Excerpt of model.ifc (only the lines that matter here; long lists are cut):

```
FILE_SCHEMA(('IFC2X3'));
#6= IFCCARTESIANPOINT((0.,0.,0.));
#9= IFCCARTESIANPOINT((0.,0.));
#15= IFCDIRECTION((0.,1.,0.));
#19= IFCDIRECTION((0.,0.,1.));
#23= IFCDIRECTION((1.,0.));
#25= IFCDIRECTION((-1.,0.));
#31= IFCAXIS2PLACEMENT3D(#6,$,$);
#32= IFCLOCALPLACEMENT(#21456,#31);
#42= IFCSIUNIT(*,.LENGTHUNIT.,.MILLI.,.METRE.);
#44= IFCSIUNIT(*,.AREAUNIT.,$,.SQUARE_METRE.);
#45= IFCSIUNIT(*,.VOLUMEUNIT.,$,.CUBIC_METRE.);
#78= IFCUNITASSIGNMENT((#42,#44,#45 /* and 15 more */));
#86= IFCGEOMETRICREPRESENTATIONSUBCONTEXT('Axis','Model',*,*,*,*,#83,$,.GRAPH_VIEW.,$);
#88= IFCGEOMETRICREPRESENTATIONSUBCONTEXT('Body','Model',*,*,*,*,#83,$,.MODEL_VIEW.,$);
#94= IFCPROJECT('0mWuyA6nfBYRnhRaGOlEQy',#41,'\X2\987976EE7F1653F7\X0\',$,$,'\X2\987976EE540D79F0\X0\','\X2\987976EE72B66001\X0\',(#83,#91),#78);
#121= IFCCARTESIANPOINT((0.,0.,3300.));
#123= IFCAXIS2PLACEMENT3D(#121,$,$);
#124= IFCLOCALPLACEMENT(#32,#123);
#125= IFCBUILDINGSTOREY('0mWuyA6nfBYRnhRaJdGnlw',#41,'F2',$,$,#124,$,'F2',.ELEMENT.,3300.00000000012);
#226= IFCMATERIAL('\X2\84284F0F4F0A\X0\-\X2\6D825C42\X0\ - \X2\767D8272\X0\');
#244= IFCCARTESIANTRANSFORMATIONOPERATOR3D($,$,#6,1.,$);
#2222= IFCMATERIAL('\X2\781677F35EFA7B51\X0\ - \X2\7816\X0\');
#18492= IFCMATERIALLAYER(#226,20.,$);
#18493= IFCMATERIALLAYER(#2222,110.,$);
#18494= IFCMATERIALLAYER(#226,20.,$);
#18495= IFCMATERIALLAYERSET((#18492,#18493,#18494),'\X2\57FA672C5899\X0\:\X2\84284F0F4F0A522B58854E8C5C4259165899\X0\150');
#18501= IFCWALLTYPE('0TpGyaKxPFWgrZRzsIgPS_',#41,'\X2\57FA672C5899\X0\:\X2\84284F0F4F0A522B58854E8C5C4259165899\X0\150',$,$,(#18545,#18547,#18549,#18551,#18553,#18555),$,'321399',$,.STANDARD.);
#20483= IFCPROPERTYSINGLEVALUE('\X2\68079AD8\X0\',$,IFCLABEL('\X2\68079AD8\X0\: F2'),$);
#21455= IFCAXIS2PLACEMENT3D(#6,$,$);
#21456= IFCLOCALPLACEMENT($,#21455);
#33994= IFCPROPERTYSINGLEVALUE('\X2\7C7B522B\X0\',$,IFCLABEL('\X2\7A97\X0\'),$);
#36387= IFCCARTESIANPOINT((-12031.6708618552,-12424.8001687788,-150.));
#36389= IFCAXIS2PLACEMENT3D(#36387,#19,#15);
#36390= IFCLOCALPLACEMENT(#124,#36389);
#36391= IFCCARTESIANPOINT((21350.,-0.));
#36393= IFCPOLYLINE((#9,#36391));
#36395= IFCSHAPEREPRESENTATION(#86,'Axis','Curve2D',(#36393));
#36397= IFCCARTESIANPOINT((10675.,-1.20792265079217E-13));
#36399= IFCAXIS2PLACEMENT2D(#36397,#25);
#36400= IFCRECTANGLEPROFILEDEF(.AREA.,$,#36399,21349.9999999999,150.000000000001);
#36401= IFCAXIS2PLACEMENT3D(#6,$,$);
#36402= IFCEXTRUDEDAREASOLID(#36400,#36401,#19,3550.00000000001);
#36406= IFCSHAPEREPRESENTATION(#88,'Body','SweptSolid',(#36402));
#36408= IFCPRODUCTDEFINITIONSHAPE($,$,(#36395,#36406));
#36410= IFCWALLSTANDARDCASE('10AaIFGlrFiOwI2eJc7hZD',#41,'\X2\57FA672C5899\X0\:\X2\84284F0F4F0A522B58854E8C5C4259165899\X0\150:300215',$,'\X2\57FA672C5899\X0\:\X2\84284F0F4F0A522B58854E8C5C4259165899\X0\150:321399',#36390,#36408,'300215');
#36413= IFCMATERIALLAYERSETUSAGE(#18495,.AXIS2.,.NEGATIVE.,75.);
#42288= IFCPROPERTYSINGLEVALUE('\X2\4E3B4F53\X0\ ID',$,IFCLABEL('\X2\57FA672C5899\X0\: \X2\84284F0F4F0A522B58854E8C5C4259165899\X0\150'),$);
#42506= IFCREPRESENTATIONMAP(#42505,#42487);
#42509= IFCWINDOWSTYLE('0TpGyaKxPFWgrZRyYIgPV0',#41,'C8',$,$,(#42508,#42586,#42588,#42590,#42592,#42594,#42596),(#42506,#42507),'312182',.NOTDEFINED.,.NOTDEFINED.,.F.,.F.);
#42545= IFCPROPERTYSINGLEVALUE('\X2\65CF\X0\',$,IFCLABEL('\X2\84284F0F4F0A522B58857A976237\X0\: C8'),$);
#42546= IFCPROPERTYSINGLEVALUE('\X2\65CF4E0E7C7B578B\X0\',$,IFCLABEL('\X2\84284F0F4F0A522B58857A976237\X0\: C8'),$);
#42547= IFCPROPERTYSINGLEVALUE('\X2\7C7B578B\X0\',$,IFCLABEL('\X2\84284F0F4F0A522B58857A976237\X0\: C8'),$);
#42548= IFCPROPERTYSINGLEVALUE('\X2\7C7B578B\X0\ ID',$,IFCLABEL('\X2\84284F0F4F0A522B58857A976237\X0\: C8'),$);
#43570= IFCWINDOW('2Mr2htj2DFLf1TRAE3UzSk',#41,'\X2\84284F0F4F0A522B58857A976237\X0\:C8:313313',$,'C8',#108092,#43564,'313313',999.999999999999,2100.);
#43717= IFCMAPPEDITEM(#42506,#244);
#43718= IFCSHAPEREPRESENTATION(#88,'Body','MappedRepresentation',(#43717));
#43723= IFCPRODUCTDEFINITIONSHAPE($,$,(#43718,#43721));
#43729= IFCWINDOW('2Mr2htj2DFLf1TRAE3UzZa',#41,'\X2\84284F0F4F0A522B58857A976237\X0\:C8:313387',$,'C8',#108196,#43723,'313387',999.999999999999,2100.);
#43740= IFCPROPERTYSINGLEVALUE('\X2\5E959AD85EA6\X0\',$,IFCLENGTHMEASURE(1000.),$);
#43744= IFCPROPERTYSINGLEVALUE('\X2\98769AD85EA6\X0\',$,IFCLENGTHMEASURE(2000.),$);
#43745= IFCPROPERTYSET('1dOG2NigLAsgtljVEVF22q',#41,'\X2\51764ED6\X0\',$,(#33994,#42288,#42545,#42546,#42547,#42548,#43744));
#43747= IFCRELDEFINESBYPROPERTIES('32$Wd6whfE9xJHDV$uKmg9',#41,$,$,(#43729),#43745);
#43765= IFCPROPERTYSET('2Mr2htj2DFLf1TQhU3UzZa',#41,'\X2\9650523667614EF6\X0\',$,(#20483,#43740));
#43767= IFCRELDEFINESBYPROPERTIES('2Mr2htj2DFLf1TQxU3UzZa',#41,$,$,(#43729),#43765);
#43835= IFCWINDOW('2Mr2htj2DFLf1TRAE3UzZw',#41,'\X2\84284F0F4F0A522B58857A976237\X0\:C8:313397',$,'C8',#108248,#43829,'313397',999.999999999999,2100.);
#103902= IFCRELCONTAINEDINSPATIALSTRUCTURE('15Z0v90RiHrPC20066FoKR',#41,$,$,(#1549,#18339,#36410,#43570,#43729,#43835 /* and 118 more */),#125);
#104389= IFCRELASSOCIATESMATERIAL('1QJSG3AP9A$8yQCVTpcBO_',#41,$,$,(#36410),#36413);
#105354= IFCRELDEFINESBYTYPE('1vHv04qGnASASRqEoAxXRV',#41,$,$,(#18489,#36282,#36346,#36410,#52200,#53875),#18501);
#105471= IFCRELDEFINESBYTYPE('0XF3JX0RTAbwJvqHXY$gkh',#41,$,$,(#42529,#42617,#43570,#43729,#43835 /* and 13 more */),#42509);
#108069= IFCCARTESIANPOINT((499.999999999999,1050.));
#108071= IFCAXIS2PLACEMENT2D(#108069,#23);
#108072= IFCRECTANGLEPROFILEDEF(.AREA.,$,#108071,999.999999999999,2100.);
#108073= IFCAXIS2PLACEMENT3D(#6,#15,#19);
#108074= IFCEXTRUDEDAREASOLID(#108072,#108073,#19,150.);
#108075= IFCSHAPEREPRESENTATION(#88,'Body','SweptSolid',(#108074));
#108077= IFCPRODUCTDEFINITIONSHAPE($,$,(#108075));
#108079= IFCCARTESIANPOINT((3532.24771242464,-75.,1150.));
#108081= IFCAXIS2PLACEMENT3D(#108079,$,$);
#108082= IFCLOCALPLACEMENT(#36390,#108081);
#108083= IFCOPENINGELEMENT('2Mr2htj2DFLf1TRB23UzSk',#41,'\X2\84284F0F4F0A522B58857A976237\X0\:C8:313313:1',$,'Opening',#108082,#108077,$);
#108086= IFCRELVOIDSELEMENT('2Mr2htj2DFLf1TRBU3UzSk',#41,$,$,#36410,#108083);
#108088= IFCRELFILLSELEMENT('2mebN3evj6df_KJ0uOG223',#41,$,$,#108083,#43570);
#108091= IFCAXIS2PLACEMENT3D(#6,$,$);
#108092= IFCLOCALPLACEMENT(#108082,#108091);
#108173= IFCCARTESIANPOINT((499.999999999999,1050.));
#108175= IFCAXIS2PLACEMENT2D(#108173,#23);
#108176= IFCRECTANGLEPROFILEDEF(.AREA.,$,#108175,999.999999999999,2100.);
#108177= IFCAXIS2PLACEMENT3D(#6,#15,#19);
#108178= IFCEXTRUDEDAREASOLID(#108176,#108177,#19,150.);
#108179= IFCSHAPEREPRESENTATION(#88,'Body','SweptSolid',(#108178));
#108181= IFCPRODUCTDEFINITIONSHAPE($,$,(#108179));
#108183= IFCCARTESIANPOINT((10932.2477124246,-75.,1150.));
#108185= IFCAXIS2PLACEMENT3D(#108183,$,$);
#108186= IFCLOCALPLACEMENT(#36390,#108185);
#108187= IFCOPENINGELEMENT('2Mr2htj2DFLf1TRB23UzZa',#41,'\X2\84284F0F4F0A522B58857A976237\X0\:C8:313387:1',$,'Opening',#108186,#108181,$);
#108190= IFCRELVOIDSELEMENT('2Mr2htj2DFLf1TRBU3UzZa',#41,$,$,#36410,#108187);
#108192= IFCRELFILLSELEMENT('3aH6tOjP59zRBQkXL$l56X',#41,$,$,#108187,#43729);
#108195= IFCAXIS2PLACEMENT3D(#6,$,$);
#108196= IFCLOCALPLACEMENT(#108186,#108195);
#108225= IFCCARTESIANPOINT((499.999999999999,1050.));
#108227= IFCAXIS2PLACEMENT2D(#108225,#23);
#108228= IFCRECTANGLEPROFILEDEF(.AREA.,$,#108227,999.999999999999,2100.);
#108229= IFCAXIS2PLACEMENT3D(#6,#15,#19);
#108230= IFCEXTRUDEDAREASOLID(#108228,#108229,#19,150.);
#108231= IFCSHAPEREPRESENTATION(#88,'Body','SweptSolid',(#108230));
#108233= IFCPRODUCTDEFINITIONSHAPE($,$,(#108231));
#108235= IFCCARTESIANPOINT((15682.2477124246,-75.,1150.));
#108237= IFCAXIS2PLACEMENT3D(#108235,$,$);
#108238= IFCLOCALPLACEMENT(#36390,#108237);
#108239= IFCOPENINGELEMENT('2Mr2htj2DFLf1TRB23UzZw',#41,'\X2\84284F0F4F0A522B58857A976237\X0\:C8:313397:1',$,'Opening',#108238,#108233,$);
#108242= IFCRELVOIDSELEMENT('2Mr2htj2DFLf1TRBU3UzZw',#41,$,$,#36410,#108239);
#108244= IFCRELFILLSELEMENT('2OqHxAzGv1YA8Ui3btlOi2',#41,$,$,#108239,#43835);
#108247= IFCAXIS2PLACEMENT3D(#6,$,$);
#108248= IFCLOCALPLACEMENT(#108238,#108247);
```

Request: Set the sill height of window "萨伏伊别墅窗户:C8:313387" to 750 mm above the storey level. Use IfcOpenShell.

```python
import numpy as np
import ifcopenshell
import ifcopenshell.api.geometry
import ifcopenshell.api.pset
import ifcopenshell.geom
import ifcopenshell.util.element
import ifcopenshell.util.placement
import ifcopenshell.util.shape
import ifcopenshell.util.unit

model = ifcopenshell.open("model.ifc")
unit_scale = ifcopenshell.util.unit.calculate_unit_scale(model)

window = model.by_guid("2Mr2htj2DFLf1TRAE3UzZa")
opening = window.FillsVoids[0].RelatingOpeningElement
storey = ifcopenshell.util.element.get_container(window, ifc_class="IfcBuildingStorey")
level = ifcopenshell.util.placement.get_local_placement(storey.ObjectPlacement)[2, 3]

# The opening's origin need not be at the sill, so measure its lowest point.
shape = ifcopenshell.geom.create_shape(ifcopenshell.geom.settings(), opening)
bottom = ifcopenshell.util.shape.get_shape_bottom_elevation(shape, shape.geometry) / unit_scale
dz = level + 750.0 - bottom

shift = np.array([0.0, 0.0, dz])
# The window is placed relative to its opening, so it follows when the opening moves.
matrix = ifcopenshell.util.placement.get_local_placement(opening.ObjectPlacement)
matrix[:3, 3] += shift
ifcopenshell.api.geometry.edit_object_placement(
    model, product=opening, matrix=matrix, is_si=False, should_transform_children=True
)

# Keep the stored heights in step.
pset = model.by_id(ifcopenshell.util.element.get_pset(window, "其他", should_inherit=False)["id"])
ifcopenshell.api.pset.edit_pset(model, pset=pset, properties={
    "顶高度": model.create_entity("IfcLengthMeasure", ifcopenshell.util.element.get_pset(window, "其他", "顶高度") + dz),
})
pset = model.by_id(ifcopenshell.util.element.get_pset(window, "限制条件", should_inherit=False)["id"])
ifcopenshell.api.pset.edit_pset(model, pset=pset, properties={
    "底高度": model.create_entity("IfcLengthMeasure", ifcopenshell.util.element.get_pset(window, "限制条件", "底高度") + dz),
})

print(f"moved by {dz * unit_scale:+.3f} m")

model.write("model_rev.ifc")
```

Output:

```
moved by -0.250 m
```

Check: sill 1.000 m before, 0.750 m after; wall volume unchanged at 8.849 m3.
